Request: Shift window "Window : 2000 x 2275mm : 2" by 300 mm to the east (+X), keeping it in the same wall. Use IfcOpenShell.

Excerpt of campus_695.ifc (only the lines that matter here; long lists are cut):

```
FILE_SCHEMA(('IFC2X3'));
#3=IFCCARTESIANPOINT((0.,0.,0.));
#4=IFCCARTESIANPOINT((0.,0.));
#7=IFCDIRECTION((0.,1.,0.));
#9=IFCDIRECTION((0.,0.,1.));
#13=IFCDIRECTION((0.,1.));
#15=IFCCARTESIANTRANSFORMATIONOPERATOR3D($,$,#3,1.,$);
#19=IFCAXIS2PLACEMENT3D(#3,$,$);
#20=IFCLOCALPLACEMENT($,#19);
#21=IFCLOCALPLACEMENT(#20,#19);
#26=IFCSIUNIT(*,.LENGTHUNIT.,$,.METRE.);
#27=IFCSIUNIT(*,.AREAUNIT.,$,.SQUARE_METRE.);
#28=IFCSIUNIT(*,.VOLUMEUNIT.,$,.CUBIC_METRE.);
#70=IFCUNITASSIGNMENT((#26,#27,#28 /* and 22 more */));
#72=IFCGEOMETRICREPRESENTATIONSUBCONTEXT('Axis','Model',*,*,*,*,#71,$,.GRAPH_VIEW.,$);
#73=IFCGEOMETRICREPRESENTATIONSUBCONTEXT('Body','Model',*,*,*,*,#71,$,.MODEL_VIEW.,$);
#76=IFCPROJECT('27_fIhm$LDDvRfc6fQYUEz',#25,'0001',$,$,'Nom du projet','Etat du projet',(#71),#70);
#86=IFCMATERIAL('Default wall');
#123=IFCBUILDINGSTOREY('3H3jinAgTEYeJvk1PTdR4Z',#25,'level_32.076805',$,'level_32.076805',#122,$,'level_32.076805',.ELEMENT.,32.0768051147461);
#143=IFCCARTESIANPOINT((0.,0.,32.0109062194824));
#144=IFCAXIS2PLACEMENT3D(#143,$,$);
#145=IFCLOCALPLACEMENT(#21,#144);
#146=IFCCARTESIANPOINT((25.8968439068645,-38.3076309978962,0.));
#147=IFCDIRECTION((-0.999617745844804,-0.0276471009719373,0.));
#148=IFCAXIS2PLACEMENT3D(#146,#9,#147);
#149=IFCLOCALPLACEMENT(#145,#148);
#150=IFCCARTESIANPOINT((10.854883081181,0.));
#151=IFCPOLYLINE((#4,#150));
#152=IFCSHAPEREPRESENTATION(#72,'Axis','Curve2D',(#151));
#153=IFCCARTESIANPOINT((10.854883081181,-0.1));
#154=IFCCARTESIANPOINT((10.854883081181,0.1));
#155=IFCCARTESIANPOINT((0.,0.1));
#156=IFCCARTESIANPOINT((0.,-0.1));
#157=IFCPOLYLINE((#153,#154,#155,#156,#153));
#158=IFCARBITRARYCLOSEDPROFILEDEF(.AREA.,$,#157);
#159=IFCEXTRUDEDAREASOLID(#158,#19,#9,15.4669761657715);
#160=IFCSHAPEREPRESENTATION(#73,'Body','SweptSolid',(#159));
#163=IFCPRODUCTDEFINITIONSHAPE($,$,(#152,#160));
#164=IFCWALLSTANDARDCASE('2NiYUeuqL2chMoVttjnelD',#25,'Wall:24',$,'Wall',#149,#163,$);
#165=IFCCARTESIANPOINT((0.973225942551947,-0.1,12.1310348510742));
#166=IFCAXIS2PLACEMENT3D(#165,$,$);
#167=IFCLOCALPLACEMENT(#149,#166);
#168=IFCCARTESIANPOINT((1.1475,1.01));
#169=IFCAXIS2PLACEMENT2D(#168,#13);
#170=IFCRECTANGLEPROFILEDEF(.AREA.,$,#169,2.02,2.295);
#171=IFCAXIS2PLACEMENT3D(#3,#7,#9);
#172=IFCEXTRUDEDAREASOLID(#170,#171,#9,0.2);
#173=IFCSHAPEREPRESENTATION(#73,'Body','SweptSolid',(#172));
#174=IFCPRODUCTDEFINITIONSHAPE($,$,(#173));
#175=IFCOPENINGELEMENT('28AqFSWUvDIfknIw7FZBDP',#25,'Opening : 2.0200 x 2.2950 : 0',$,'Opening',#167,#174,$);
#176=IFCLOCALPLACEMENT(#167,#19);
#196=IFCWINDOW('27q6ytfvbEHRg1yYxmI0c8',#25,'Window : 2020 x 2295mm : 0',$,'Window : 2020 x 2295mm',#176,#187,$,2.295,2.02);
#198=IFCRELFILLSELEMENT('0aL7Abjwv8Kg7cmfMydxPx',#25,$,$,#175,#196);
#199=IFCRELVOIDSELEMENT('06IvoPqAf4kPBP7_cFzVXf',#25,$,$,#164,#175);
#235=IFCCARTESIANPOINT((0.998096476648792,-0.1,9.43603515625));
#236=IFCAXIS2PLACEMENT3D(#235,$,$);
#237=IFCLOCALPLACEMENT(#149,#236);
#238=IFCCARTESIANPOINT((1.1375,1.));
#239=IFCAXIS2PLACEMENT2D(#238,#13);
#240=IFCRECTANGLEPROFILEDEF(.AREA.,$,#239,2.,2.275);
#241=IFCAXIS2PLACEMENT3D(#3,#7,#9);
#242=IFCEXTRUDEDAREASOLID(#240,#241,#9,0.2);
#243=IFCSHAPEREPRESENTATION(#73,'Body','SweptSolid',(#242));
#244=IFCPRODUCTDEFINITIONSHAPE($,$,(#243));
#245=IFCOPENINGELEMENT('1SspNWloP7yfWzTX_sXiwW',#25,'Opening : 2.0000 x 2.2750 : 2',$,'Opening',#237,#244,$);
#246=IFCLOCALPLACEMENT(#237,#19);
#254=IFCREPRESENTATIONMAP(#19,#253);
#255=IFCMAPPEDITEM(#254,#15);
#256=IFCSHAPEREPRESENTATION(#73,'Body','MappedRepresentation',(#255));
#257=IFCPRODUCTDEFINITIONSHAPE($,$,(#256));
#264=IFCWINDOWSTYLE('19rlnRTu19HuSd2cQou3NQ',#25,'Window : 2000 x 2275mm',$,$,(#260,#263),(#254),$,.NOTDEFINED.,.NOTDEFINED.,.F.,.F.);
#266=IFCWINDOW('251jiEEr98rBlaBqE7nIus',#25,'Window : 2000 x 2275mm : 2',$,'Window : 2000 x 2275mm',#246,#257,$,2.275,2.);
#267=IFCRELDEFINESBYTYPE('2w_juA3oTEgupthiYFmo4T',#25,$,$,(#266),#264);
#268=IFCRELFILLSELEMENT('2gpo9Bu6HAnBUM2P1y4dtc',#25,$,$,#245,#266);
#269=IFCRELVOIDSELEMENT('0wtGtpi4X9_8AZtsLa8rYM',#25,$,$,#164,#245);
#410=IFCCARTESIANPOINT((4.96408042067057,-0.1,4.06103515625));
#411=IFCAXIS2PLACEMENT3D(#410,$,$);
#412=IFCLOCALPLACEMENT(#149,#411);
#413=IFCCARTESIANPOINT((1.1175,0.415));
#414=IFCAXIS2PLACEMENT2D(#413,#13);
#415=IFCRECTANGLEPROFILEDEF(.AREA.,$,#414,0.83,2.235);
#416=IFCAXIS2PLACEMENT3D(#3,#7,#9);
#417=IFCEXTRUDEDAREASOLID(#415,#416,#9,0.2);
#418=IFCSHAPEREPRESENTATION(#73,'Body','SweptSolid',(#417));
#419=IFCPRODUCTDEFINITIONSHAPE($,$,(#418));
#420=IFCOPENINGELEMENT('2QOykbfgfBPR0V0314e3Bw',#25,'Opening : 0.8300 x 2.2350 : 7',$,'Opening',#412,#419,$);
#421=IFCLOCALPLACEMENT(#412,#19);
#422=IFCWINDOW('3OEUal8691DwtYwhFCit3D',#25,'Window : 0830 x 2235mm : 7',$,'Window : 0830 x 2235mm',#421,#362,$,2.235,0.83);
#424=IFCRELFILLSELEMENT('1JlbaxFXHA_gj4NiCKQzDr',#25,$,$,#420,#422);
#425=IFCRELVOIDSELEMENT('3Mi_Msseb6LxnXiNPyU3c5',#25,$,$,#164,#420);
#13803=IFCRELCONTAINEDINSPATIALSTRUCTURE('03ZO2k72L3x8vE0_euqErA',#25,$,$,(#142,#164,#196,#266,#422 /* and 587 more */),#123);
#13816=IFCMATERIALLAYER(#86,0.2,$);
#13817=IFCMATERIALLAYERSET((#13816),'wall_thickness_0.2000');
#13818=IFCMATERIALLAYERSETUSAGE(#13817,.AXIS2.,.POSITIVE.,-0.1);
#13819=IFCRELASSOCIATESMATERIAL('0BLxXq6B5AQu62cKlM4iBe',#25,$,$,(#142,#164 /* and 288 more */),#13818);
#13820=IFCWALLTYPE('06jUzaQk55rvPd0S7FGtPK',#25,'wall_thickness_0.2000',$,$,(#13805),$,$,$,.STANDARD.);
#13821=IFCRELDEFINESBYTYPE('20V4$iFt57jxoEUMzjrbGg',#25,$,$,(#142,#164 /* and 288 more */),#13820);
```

```python
import ifcopenshell
import ifcopenshell.api.geometry
import ifcopenshell.util.placement
import ifcopenshell.util.unit

model = ifcopenshell.open("campus_695.ifc")
unit_scale = ifcopenshell.util.unit.calculate_unit_scale(model)

window = model.by_guid("251jiEEr98rBlaBqE7nIus")
opening = window.FillsVoids[0].RelatingOpeningElement
wall = opening.VoidsElements[0].RelatingBuildingElement

wall_matrix = ifcopenshell.util.placement.get_local_placement(wall.ObjectPlacement)
shift = wall_matrix[:3, 0] * -0.3 / unit_scale
before = ifcopenshell.util.placement.get_local_placement(window.ObjectPlacement)[:3, 3].copy()

# The window is placed relative to its opening, so it follows when the opening moves.
matrix = ifcopenshell.util.placement.get_local_placement(opening.ObjectPlacement)
matrix[:3, 3] += shift
ifcopenshell.api.geometry.edit_object_placement(
    model, product=opening, matrix=matrix, is_si=False, should_transform_children=True
)

after = ifcopenshell.util.placement.get_local_placement(window.ObjectPlacement)[:3, 3]
print("window moved by", (after - before).round(3) + 0.0)

model.write("campus_695_rev.ifc")
```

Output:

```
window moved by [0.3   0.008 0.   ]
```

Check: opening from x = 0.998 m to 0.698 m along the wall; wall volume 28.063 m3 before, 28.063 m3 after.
